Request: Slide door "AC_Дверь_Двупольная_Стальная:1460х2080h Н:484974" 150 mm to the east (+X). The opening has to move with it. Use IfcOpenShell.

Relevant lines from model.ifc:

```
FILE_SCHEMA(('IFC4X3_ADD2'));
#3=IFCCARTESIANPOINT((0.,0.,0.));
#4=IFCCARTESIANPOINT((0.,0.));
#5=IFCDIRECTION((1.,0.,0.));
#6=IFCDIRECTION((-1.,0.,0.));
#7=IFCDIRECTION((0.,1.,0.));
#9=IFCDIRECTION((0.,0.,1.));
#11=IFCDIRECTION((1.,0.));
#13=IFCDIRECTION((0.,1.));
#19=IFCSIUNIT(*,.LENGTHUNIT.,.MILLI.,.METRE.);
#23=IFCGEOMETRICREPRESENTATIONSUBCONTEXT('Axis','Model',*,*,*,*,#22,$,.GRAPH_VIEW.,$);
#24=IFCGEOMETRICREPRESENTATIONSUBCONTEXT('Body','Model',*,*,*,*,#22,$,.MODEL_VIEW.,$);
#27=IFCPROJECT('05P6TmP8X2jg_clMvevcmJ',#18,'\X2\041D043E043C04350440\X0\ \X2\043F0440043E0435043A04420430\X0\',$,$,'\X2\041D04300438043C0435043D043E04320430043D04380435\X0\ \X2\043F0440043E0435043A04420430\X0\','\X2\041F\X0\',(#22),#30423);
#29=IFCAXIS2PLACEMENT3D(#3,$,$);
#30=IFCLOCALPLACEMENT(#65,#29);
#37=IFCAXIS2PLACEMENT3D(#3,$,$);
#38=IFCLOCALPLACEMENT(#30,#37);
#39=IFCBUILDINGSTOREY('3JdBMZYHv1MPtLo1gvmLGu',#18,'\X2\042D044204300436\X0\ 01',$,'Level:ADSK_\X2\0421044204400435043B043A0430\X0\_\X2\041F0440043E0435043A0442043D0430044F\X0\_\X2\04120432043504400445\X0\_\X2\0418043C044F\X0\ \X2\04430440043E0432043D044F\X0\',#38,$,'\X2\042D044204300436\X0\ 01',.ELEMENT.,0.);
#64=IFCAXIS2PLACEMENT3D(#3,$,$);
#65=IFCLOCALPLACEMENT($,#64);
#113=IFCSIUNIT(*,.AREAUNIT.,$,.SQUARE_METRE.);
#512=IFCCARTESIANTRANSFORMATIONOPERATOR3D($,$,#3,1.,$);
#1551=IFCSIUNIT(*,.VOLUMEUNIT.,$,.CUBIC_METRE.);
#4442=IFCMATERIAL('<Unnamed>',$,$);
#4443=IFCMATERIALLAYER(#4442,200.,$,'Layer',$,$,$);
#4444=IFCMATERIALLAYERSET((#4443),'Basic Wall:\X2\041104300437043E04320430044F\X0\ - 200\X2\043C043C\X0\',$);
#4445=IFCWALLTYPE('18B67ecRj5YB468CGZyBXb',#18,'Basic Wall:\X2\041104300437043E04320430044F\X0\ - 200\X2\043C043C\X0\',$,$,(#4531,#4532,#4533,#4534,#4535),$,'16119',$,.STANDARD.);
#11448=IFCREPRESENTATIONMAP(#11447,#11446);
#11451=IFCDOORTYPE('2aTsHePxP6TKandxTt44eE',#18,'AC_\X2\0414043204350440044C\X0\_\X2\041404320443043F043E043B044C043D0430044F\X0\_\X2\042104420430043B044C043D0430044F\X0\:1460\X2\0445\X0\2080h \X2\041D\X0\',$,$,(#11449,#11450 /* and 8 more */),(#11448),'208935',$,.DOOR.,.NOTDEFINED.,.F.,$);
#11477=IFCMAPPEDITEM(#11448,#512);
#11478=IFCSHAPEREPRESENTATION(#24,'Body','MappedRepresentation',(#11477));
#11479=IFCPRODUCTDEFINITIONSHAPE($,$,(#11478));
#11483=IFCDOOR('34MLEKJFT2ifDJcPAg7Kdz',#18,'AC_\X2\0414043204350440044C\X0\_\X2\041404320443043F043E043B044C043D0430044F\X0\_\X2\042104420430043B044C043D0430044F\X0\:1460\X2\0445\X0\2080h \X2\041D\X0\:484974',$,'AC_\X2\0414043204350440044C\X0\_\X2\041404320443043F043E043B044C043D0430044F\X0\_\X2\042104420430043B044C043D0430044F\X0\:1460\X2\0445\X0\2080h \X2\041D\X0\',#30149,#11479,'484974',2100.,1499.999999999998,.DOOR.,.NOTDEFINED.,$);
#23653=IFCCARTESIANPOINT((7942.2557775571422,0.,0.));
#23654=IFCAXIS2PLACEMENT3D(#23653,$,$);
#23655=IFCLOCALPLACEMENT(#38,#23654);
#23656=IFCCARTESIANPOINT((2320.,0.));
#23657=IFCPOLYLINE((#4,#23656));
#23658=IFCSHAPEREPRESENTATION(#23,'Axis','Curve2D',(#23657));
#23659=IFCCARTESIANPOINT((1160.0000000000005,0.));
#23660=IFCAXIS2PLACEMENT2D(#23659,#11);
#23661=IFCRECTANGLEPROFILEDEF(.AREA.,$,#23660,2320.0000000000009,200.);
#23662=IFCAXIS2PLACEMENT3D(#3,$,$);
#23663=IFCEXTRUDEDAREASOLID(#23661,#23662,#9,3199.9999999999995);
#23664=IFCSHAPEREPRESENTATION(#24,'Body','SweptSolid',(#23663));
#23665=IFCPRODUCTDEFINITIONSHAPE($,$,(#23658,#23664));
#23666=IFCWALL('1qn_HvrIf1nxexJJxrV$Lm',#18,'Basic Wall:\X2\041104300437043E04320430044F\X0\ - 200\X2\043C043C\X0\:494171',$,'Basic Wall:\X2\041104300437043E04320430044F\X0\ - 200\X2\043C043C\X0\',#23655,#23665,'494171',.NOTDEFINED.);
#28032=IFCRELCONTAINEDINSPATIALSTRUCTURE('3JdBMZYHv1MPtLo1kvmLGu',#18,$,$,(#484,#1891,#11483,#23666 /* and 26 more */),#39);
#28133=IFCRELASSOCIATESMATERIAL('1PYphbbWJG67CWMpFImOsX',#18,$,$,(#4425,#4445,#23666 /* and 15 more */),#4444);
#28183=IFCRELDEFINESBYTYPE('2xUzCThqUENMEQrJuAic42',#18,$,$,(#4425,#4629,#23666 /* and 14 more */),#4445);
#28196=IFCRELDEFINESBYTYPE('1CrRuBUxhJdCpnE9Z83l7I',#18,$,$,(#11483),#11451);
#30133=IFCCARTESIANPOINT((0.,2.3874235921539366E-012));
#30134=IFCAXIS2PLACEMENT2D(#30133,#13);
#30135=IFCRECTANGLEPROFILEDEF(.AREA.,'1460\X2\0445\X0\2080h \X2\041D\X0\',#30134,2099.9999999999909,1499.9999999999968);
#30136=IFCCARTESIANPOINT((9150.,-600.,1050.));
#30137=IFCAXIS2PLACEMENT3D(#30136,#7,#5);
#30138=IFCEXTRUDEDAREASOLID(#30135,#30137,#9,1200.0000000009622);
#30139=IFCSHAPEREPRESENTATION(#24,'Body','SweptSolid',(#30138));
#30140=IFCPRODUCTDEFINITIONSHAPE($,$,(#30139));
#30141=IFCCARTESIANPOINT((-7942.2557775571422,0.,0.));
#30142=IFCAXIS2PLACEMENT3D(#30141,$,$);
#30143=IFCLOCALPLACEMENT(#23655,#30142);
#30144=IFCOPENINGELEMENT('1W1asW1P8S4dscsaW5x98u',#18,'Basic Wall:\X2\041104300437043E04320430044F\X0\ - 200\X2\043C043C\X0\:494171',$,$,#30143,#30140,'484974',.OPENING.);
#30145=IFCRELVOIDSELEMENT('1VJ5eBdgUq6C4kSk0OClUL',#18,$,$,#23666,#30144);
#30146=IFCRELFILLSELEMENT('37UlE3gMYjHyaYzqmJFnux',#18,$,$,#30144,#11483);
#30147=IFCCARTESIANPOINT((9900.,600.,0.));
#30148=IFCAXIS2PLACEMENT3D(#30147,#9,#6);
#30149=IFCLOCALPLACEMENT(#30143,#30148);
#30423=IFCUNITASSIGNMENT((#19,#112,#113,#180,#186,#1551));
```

```python
import ifcopenshell
import ifcopenshell.api.geometry
import ifcopenshell.util.placement

model = ifcopenshell.open("model.ifc")

door = model.by_guid("34MLEKJFT2ifDJcPAg7Kdz")
opening = door.FillsVoids[0].RelatingOpeningElement
wall = opening.VoidsElements[0].RelatingBuildingElement

wall_matrix = ifcopenshell.util.placement.get_local_placement(wall.ObjectPlacement)
shift = wall_matrix[:3, 0] * 150.0
before = ifcopenshell.util.placement.get_local_placement(door.ObjectPlacement)[:3, 3].copy()

# The door is placed relative to its opening, so it follows when the opening moves.
matrix = ifcopenshell.util.placement.get_local_placement(opening.ObjectPlacement)
matrix[:3, 3] += shift
ifcopenshell.api.geometry.edit_object_placement(
    model, product=opening, matrix=matrix, is_si=False, should_transform_children=True
)

after = ifcopenshell.util.placement.get_local_placement(door.ObjectPlacement)[:3, 3]
print("door moved by", (after - before).round(3) + 0.0)

model.write("model-out.ifc")
```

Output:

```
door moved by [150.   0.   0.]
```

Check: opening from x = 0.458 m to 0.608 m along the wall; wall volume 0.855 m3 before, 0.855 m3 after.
